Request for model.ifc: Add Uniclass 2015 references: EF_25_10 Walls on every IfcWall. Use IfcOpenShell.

First a look at what the model holds.

```python
import ifcopenshell

model = ifcopenshell.open("model.ifc")
print(model.schema)
print("classifications:", [c.Name for c in model.by_type("IfcClassification")])
for ifc_class in ("IfcDoor", "IfcRoof", "IfcStair", "IfcWall", "IfcWindow"):
    print(ifc_class, len(model.by_type(ifc_class)))
```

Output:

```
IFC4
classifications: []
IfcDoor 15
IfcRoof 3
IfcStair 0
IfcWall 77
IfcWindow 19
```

```python
import ifcopenshell
import ifcopenshell.api.classification

model = ifcopenshell.open("model.ifc")

system = ifcopenshell.api.classification.add_classification(model, classification="Uniclass 2015")

codes = {
    "IfcWall": ("EF_25_10", "Walls"),
}
for ifc_class, (code, name) in codes.items():
    products = model.by_type(ifc_class)
    ifcopenshell.api.classification.add_reference(
        model, products=products, classification=system, identification=code, name=name
    )
    print(code, len(products))

model.write("model_updated.ifc")
```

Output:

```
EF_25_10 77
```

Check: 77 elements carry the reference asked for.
